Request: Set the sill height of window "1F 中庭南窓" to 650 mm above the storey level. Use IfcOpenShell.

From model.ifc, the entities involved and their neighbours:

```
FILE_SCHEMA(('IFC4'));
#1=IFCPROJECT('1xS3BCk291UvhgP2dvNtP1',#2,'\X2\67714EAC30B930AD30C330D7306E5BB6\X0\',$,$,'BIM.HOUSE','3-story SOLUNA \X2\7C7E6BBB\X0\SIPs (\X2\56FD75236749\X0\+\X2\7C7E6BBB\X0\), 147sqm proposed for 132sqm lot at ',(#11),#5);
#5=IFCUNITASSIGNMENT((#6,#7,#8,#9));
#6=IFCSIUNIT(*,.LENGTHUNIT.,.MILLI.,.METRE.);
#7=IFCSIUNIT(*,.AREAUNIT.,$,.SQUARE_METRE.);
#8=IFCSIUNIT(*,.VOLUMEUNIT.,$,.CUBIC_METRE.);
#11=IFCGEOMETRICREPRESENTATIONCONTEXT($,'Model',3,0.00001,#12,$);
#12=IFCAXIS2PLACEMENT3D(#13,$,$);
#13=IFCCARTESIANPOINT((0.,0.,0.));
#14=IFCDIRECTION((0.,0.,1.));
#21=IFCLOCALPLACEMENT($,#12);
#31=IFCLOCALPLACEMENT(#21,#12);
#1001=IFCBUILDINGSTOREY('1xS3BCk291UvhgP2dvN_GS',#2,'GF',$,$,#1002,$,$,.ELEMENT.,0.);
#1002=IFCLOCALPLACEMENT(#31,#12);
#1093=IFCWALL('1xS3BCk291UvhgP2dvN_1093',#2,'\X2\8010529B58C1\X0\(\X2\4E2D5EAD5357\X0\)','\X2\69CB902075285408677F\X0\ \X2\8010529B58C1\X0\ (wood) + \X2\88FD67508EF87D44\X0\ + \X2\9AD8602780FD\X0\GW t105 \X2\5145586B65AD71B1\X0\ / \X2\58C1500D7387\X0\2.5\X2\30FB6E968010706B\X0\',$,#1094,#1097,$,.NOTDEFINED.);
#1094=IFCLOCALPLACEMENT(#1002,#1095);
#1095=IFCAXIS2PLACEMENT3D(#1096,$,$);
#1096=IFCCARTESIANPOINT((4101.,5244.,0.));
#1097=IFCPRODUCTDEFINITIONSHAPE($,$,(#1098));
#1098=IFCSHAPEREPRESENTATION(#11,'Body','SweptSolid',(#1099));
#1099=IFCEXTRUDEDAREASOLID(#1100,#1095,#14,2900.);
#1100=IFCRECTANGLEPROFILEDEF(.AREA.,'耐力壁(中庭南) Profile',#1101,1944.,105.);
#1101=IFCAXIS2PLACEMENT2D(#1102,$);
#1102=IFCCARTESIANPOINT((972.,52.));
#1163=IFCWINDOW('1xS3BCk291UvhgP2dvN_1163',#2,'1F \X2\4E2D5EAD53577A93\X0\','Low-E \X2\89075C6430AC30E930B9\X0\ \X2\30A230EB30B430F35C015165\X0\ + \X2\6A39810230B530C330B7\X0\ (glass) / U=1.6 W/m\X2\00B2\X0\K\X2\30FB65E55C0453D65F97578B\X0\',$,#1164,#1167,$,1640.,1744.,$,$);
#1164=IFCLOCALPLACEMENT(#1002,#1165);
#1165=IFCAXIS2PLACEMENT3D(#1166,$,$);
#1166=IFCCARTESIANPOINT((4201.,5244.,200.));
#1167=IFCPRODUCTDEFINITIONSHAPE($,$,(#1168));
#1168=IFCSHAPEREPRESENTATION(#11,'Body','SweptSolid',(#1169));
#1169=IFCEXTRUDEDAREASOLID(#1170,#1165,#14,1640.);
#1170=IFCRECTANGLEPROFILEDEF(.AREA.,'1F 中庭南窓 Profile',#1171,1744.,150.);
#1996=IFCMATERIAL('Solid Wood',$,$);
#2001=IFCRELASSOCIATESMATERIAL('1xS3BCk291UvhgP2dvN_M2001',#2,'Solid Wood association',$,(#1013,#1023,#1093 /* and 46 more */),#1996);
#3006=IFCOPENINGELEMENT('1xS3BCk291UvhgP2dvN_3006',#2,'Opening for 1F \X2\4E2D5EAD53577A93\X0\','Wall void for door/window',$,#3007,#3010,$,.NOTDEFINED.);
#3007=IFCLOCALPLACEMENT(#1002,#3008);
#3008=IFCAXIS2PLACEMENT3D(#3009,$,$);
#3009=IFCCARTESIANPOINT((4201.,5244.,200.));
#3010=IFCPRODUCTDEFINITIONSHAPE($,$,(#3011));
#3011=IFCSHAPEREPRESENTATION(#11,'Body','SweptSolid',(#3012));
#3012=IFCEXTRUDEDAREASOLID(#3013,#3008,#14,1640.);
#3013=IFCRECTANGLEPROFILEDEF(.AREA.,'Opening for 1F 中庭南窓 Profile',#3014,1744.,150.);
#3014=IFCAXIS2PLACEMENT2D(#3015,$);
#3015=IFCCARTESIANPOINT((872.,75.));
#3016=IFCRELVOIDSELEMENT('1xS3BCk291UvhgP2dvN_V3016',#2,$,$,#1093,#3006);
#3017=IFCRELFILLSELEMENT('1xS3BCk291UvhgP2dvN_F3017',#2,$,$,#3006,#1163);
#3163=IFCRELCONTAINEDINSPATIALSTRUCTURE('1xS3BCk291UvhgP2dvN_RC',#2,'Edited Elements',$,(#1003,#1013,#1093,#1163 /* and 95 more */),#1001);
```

```python
import numpy as np
import ifcopenshell
import ifcopenshell.api.geometry
import ifcopenshell.geom
import ifcopenshell.util.element
import ifcopenshell.util.placement
import ifcopenshell.util.shape
import ifcopenshell.util.unit

model = ifcopenshell.open("model.ifc")
unit_scale = ifcopenshell.util.unit.calculate_unit_scale(model)

window = model.by_id(1163)
opening = window.FillsVoids[0].RelatingOpeningElement
storey = ifcopenshell.util.element.get_container(window, ifc_class="IfcBuildingStorey")
level = ifcopenshell.util.placement.get_local_placement(storey.ObjectPlacement)[2, 3]

# The opening's origin need not be at the sill, so measure its lowest point.
shape = ifcopenshell.geom.create_shape(ifcopenshell.geom.settings(), opening)
bottom = ifcopenshell.util.shape.get_shape_bottom_elevation(shape, shape.geometry) / unit_scale
dz = level + 0.65 / unit_scale - bottom

shift = np.array([0.0, 0.0, dz])
# The window is not placed relative to its opening, so move both.
for product in (opening, window):
    matrix = ifcopenshell.util.placement.get_local_placement(product.ObjectPlacement)
    matrix[:3, 3] += shift
    ifcopenshell.api.geometry.edit_object_placement(model, product=product, matrix=matrix, is_si=False)

print(f"moved by {dz * unit_scale:+.3f} m")

model.write("model-out.ifc")
```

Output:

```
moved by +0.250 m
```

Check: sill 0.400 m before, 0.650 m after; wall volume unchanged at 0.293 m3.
